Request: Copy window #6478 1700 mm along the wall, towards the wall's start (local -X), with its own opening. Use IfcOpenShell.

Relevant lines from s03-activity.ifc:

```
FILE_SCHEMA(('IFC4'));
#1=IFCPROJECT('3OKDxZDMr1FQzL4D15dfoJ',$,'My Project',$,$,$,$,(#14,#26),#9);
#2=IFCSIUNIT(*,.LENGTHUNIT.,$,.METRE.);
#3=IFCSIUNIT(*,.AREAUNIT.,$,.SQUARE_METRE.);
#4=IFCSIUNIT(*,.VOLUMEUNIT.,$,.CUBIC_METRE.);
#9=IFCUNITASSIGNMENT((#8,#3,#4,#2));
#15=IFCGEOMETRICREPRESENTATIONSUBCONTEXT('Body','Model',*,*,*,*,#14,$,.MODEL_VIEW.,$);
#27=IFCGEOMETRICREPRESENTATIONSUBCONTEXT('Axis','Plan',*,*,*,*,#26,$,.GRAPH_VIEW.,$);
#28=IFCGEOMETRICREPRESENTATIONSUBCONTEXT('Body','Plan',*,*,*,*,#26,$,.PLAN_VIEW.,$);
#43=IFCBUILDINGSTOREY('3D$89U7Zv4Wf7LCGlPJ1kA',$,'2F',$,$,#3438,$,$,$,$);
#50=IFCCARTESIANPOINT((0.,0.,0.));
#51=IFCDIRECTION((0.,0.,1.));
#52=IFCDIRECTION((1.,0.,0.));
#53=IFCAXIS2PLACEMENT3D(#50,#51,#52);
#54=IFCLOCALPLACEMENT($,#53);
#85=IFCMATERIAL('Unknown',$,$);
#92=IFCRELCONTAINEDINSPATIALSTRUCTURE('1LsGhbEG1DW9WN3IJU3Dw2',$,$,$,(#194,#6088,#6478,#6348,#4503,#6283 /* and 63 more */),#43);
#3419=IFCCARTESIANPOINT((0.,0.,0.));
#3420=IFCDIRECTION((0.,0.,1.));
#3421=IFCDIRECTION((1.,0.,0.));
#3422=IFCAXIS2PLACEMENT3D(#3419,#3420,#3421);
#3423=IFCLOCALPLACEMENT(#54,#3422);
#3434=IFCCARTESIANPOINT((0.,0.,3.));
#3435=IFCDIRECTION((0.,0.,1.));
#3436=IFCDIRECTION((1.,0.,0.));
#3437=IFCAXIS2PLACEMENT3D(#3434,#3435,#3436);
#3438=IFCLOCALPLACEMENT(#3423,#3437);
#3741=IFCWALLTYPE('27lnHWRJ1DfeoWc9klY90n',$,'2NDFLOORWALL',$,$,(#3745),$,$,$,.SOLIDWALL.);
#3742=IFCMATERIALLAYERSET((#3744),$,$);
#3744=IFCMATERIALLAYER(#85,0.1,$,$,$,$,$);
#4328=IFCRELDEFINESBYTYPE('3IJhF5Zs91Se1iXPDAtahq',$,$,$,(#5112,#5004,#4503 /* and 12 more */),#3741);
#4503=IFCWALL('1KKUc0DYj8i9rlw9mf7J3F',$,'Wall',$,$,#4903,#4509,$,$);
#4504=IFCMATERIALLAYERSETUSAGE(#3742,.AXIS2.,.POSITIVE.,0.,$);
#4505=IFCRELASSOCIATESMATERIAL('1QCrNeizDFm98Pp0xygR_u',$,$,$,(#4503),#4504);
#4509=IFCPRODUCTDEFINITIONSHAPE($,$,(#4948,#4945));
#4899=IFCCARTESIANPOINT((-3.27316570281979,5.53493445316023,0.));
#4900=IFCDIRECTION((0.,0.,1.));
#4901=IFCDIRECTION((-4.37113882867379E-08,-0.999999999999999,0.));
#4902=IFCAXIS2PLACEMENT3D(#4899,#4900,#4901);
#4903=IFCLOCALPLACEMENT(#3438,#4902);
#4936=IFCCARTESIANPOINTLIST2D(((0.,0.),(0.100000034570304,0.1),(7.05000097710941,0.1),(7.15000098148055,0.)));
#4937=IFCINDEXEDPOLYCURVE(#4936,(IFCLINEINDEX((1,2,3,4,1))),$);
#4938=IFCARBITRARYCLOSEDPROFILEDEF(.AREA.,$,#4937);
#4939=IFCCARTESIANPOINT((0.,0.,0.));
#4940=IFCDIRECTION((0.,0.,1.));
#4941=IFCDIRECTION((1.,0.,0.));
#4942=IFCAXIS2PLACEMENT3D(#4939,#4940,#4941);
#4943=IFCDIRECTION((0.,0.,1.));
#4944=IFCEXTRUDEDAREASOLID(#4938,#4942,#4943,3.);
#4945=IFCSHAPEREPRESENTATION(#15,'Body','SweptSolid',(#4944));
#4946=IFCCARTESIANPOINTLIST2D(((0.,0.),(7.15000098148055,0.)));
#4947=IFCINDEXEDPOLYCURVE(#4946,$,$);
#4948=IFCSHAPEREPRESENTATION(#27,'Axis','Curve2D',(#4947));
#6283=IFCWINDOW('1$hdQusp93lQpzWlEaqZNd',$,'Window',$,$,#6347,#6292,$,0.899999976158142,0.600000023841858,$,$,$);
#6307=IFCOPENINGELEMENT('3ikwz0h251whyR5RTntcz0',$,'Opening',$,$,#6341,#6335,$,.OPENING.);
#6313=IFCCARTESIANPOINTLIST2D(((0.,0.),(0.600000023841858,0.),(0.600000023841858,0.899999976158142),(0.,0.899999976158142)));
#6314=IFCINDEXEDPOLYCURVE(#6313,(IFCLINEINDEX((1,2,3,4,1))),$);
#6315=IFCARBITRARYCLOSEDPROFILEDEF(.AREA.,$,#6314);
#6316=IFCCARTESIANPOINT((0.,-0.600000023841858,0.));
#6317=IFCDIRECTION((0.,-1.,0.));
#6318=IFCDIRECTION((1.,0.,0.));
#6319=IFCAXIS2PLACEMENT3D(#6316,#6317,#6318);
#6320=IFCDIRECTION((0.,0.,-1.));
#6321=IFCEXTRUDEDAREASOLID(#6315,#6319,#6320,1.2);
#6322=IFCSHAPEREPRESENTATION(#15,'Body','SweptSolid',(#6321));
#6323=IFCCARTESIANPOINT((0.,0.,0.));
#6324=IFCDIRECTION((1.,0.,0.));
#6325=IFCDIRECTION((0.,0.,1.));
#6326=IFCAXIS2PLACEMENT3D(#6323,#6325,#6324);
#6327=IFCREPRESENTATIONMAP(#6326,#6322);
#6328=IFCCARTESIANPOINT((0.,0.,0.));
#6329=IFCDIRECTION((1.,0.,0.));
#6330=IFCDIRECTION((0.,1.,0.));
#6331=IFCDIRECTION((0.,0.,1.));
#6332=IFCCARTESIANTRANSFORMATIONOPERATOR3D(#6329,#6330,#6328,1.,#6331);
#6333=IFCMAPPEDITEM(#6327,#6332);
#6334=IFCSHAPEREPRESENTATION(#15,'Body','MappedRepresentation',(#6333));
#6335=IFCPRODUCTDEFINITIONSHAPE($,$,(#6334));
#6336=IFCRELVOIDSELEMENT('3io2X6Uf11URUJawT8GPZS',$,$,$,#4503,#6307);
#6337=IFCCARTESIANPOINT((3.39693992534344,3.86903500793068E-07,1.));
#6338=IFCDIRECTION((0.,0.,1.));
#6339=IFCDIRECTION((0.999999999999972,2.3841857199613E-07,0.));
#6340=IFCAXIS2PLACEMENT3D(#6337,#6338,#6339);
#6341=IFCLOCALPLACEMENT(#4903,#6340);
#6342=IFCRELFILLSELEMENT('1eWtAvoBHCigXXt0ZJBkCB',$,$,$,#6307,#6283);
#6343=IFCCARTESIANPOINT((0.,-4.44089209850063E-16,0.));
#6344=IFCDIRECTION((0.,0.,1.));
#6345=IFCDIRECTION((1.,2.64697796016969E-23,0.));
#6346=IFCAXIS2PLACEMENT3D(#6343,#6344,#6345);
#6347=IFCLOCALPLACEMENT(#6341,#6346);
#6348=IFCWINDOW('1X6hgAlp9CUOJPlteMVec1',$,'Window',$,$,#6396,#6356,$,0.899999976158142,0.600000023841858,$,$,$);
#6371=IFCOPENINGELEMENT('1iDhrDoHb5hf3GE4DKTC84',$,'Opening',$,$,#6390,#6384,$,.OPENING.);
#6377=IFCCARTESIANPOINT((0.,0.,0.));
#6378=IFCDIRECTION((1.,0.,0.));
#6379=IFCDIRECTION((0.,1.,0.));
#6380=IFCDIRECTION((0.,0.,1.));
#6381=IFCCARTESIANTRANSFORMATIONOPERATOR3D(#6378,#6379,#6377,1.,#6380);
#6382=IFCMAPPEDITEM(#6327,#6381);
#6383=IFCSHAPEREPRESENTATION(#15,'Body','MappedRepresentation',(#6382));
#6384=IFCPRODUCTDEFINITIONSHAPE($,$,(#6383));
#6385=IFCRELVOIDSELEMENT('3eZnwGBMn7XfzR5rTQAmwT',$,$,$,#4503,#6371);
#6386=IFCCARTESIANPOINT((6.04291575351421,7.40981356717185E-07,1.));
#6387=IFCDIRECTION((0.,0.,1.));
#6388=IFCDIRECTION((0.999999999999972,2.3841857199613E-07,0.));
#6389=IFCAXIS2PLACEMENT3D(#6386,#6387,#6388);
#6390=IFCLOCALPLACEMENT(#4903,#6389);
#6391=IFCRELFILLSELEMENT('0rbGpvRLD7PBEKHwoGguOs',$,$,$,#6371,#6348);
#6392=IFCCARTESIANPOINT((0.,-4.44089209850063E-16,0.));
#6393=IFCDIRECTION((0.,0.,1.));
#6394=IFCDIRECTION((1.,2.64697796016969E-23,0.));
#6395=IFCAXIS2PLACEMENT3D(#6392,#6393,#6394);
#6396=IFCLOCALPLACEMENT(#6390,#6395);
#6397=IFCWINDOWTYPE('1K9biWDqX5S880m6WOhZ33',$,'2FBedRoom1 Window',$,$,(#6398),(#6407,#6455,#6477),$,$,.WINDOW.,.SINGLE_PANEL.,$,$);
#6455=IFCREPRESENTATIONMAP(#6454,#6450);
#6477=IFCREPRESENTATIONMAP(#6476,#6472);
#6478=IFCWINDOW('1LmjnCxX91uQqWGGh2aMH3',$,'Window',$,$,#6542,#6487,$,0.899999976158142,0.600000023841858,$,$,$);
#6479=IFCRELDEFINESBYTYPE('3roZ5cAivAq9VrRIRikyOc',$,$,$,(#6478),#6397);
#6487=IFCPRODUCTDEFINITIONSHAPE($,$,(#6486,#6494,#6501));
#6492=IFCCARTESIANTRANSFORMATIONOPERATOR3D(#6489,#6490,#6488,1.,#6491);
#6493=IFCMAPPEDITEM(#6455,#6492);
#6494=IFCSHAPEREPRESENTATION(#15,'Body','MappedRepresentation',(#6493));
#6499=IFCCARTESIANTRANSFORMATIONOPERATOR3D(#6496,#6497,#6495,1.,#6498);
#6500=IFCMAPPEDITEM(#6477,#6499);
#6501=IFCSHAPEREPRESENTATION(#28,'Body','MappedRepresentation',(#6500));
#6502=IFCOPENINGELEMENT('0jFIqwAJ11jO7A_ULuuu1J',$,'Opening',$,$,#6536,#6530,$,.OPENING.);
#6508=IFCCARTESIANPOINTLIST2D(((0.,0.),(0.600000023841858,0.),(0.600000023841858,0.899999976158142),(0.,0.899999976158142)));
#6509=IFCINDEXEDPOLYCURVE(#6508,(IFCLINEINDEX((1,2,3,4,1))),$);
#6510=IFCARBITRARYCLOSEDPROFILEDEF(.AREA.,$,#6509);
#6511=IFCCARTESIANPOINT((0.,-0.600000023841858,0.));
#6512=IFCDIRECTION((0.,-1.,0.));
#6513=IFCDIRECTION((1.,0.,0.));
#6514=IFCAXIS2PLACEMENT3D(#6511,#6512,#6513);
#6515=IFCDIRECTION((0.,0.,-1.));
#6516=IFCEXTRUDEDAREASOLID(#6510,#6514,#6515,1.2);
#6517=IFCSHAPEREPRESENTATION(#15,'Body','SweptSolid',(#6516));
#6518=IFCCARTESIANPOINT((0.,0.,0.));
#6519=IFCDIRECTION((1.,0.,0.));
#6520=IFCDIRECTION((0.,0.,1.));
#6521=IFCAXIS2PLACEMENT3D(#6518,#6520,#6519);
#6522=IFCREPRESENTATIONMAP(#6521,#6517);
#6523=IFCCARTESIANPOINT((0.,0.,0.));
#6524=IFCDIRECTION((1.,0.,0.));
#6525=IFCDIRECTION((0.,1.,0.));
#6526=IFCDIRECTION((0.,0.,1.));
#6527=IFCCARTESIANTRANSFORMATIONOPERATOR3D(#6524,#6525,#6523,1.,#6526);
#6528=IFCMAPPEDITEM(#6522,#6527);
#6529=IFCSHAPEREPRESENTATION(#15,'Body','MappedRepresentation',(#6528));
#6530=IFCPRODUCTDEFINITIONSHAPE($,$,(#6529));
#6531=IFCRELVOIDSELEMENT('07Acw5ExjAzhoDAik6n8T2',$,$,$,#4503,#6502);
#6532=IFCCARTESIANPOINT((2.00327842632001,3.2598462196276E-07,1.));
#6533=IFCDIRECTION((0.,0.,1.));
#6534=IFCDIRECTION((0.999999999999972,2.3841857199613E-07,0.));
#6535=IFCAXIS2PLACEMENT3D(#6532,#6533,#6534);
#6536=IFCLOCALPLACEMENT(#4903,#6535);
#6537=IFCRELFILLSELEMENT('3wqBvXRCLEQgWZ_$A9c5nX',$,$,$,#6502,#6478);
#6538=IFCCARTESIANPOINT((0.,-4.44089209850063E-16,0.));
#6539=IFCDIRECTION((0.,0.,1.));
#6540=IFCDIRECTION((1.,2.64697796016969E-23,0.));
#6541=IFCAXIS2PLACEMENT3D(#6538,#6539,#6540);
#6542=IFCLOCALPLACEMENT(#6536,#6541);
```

```python
import ifcopenshell
import ifcopenshell.api.feature
import ifcopenshell.api.geometry
import ifcopenshell.api.root
import ifcopenshell.geom
import ifcopenshell.util.element
import ifcopenshell.util.placement
import ifcopenshell.util.shape
import ifcopenshell.util.unit

model = ifcopenshell.open("s03-activity.ifc")
unit_scale = ifcopenshell.util.unit.calculate_unit_scale(model)
settings = ifcopenshell.geom.settings()


def volume(element):
    """Net volume in cubic metres, openings subtracted."""
    shape = ifcopenshell.geom.create_shape(settings, element)
    return ifcopenshell.util.shape.get_volume(shape.geometry)


window = model.by_id(6478)
opening = window.FillsVoids[0].RelatingOpeningElement
wall = opening.VoidsElements[0].RelatingBuildingElement
before = volume(wall)
shift = ifcopenshell.util.placement.get_local_placement(wall.ObjectPlacement)[:3, 0] * -1.7 / unit_scale

# copy_class copies the void relationship, type, container and properties, but no geometry.
new_opening = ifcopenshell.api.root.copy_class(model, product=opening)
new_opening.Representation = ifcopenshell.util.element.copy_deep(
    model, opening.Representation, exclude=["IfcGeometricRepresentationContext", "IfcRepresentationMap"]
)
new_window = ifcopenshell.api.root.copy_class(model, product=window)
new_window.Representation = ifcopenshell.util.element.copy_deep(
    model, window.Representation, exclude=["IfcGeometricRepresentationContext", "IfcRepresentationMap"]
)
ifcopenshell.api.feature.add_filling(model, opening=new_opening, element=new_window)

for old, new in ((opening, new_opening), (window, new_window)):
    matrix = ifcopenshell.util.placement.get_local_placement(old.ObjectPlacement)
    matrix[:3, 3] += shift
    ifcopenshell.api.geometry.edit_object_placement(model, product=new, matrix=matrix, is_si=False)

after = volume(wall)

print(f"wall volume {before:.3f} -> {after:.3f} m3")

model.write("s03-activity_updated.ifc")
```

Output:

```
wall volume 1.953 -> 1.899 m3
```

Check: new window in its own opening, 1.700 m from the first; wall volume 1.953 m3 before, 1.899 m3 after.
